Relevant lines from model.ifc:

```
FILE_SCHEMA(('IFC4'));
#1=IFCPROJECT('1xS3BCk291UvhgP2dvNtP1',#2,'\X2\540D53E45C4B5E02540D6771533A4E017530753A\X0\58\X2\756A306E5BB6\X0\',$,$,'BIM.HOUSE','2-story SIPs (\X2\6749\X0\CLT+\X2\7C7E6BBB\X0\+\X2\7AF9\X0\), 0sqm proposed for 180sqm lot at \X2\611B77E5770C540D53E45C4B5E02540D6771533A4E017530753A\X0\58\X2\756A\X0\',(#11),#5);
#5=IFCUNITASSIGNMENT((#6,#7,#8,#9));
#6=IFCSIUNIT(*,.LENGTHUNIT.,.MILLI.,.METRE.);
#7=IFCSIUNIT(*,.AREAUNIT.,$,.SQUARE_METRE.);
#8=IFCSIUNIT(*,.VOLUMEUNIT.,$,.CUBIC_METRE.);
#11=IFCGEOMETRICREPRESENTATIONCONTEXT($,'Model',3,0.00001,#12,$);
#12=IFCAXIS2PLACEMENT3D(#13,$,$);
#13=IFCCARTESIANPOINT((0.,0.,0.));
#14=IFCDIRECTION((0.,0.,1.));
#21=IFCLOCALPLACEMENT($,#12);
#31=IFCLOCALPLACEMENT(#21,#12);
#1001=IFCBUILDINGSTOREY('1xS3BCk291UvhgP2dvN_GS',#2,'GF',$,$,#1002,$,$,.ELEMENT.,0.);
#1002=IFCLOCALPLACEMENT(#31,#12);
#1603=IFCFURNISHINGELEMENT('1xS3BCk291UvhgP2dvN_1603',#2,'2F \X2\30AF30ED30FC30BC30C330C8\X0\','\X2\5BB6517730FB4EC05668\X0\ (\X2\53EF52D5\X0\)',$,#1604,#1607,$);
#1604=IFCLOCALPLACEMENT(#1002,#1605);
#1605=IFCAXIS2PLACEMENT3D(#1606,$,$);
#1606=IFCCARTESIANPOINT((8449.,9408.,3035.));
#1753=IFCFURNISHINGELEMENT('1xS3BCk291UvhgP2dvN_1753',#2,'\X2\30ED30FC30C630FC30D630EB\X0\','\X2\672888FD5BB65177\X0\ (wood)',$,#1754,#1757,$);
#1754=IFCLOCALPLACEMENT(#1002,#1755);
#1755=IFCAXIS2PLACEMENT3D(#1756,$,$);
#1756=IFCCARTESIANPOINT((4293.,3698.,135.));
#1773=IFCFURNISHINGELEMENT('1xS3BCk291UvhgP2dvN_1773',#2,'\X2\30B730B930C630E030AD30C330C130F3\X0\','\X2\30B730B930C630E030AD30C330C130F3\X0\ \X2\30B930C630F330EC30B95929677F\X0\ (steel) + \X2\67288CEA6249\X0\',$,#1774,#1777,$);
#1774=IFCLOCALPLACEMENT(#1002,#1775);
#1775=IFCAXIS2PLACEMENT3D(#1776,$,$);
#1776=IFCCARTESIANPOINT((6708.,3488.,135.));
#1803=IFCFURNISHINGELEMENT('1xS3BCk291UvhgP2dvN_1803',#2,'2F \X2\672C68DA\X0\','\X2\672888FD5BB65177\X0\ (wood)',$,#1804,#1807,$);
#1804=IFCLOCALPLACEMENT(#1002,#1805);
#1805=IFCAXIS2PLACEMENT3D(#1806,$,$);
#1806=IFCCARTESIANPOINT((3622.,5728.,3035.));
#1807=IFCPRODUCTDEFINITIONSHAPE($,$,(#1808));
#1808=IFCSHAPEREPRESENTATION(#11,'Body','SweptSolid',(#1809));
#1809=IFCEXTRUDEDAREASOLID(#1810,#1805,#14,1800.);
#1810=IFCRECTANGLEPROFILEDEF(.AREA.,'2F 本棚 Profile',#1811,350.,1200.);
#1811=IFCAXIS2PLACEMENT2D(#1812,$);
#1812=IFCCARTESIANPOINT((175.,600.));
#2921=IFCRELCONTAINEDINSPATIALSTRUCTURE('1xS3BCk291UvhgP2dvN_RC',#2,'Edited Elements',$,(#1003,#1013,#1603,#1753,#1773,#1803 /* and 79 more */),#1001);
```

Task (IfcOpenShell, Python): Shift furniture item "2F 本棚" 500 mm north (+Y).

```python
import ifcopenshell
import ifcopenshell.api.geometry
import ifcopenshell.util.placement
import ifcopenshell.util.unit

model = ifcopenshell.open("model.ifc")
unit_scale = ifcopenshell.util.unit.calculate_unit_scale(model)

item = model.by_guid("1xS3BCk291UvhgP2dvN_1803")
matrix = ifcopenshell.util.placement.get_local_placement(item.ObjectPlacement)
matrix[1, 3] += 0.5 / unit_scale
ifcopenshell.api.geometry.edit_object_placement(model, product=item, matrix=matrix, is_si=False)

print(ifcopenshell.util.placement.get_local_placement(item.ObjectPlacement).round(3) + 0.0)

model.write("model-out.ifc")
```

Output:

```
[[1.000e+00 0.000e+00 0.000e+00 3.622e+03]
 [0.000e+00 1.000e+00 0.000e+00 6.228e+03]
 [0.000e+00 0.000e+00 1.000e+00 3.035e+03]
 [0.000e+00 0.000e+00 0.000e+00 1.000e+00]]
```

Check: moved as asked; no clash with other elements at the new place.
